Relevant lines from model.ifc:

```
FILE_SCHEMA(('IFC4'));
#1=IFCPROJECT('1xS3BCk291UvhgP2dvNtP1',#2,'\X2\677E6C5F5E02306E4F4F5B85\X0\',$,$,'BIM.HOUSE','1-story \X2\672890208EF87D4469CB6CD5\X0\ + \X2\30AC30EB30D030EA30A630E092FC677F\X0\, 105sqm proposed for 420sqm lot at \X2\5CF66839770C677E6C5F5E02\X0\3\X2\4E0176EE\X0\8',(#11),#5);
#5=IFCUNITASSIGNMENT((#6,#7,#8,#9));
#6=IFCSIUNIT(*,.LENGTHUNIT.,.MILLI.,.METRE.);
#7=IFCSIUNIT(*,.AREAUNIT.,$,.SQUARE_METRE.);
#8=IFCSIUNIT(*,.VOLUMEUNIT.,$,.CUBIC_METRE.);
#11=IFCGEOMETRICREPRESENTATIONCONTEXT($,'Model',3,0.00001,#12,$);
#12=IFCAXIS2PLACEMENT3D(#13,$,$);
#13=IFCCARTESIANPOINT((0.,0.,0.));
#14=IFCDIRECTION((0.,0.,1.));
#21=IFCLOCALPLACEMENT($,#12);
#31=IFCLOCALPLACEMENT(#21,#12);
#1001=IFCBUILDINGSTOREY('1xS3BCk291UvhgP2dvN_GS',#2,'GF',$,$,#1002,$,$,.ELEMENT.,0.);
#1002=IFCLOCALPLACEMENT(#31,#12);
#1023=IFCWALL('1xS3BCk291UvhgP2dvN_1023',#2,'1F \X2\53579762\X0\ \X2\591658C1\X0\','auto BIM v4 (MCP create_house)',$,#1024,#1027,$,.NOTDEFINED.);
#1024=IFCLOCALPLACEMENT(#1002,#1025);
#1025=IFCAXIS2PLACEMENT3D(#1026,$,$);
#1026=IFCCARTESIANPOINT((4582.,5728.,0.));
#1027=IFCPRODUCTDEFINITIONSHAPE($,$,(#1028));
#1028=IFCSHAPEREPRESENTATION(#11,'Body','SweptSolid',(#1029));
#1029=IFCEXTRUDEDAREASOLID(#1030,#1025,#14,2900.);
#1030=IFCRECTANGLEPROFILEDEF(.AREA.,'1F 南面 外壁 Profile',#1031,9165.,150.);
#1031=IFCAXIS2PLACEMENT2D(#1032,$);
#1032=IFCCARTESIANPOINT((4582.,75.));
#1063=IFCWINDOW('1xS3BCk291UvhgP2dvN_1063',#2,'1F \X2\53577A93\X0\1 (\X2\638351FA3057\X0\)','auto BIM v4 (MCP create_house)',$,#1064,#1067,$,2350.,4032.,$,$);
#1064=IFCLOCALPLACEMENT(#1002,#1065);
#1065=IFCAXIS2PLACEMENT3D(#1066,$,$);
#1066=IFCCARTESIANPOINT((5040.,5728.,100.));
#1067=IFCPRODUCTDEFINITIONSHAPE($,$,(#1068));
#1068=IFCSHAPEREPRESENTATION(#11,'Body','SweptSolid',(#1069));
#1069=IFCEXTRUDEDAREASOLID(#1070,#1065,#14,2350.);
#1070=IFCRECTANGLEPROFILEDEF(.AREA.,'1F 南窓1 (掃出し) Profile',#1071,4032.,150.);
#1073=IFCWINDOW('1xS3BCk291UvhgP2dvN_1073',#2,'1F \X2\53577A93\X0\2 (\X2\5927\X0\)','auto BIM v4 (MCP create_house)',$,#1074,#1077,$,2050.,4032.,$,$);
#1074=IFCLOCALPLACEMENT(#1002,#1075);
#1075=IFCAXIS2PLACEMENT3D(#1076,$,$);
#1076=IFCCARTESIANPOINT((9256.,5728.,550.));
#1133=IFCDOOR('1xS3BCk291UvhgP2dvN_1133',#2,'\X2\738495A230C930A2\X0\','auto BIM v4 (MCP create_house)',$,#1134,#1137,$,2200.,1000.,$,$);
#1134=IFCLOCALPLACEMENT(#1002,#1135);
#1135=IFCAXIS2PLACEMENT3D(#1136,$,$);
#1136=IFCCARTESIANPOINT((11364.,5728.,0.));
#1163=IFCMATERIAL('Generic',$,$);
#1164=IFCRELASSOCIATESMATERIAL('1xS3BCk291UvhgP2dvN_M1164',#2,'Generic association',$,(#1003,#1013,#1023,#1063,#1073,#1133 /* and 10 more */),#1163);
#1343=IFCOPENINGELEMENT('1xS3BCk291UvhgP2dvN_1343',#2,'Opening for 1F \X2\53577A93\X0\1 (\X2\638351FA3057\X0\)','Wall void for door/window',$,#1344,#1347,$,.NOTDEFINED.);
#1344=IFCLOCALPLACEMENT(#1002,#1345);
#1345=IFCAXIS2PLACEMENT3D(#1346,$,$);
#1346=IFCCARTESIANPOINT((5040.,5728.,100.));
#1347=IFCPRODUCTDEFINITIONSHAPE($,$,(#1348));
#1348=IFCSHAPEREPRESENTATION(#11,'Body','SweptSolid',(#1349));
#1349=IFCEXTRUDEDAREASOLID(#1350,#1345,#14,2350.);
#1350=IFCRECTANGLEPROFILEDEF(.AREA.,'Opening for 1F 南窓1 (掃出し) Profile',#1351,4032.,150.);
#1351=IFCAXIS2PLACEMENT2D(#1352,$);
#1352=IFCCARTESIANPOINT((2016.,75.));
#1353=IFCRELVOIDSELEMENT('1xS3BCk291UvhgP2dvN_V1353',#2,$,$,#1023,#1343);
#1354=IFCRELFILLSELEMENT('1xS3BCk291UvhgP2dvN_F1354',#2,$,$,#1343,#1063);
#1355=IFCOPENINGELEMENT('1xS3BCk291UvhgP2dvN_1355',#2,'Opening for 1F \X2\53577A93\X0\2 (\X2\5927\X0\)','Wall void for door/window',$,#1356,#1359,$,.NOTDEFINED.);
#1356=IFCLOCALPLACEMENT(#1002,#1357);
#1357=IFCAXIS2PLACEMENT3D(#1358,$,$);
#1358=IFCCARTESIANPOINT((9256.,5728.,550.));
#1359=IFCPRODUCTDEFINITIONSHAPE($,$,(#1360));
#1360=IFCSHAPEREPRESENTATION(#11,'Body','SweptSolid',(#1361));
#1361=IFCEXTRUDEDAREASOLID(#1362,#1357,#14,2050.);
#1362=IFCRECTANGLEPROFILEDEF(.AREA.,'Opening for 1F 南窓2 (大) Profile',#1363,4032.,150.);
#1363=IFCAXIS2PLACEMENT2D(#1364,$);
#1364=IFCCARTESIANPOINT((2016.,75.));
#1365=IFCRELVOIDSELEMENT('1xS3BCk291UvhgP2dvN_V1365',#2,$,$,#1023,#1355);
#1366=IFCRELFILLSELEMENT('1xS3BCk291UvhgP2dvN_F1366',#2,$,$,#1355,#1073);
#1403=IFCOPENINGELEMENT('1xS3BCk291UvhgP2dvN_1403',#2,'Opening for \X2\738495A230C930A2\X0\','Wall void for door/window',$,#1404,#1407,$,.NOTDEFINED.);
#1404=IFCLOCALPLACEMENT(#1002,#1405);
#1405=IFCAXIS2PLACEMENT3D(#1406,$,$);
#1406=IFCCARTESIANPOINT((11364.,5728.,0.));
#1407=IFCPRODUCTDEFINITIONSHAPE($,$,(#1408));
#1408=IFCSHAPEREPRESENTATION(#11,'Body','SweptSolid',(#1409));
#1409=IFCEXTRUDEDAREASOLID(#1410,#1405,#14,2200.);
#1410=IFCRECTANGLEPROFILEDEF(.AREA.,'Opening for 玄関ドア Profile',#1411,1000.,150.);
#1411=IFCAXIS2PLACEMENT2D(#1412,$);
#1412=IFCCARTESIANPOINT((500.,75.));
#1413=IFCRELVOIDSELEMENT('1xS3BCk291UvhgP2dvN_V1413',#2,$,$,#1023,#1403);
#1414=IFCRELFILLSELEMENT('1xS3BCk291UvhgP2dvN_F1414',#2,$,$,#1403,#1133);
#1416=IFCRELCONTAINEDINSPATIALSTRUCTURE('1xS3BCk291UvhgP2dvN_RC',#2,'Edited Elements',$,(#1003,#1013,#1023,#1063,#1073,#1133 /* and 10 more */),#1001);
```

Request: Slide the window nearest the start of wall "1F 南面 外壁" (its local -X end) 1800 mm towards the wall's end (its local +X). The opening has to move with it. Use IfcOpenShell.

```python
import ifcopenshell
import ifcopenshell.api.geometry
import ifcopenshell.util.placement
import ifcopenshell.util.unit

model = ifcopenshell.open("model.ifc")
unit_scale = ifcopenshell.util.unit.calculate_unit_scale(model)

window = model.by_id(1063)
opening = window.FillsVoids[0].RelatingOpeningElement
wall = opening.VoidsElements[0].RelatingBuildingElement

wall_matrix = ifcopenshell.util.placement.get_local_placement(wall.ObjectPlacement)
shift = wall_matrix[:3, 0] * 1.8 / unit_scale
before = ifcopenshell.util.placement.get_local_placement(window.ObjectPlacement)[:3, 3].copy()

# The window is not placed relative to its opening, so move both.
for product in (opening, window):
    matrix = ifcopenshell.util.placement.get_local_placement(product.ObjectPlacement)
    matrix[:3, 3] += shift
    ifcopenshell.api.geometry.edit_object_placement(model, product=product, matrix=matrix, is_si=False)

after = ifcopenshell.util.placement.get_local_placement(window.ObjectPlacement)[:3, 3]
print("window moved by", (after - before).round(3) + 0.0)

model.write("model_edited.ifc")
```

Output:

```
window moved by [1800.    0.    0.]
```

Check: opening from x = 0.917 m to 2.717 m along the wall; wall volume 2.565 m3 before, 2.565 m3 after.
